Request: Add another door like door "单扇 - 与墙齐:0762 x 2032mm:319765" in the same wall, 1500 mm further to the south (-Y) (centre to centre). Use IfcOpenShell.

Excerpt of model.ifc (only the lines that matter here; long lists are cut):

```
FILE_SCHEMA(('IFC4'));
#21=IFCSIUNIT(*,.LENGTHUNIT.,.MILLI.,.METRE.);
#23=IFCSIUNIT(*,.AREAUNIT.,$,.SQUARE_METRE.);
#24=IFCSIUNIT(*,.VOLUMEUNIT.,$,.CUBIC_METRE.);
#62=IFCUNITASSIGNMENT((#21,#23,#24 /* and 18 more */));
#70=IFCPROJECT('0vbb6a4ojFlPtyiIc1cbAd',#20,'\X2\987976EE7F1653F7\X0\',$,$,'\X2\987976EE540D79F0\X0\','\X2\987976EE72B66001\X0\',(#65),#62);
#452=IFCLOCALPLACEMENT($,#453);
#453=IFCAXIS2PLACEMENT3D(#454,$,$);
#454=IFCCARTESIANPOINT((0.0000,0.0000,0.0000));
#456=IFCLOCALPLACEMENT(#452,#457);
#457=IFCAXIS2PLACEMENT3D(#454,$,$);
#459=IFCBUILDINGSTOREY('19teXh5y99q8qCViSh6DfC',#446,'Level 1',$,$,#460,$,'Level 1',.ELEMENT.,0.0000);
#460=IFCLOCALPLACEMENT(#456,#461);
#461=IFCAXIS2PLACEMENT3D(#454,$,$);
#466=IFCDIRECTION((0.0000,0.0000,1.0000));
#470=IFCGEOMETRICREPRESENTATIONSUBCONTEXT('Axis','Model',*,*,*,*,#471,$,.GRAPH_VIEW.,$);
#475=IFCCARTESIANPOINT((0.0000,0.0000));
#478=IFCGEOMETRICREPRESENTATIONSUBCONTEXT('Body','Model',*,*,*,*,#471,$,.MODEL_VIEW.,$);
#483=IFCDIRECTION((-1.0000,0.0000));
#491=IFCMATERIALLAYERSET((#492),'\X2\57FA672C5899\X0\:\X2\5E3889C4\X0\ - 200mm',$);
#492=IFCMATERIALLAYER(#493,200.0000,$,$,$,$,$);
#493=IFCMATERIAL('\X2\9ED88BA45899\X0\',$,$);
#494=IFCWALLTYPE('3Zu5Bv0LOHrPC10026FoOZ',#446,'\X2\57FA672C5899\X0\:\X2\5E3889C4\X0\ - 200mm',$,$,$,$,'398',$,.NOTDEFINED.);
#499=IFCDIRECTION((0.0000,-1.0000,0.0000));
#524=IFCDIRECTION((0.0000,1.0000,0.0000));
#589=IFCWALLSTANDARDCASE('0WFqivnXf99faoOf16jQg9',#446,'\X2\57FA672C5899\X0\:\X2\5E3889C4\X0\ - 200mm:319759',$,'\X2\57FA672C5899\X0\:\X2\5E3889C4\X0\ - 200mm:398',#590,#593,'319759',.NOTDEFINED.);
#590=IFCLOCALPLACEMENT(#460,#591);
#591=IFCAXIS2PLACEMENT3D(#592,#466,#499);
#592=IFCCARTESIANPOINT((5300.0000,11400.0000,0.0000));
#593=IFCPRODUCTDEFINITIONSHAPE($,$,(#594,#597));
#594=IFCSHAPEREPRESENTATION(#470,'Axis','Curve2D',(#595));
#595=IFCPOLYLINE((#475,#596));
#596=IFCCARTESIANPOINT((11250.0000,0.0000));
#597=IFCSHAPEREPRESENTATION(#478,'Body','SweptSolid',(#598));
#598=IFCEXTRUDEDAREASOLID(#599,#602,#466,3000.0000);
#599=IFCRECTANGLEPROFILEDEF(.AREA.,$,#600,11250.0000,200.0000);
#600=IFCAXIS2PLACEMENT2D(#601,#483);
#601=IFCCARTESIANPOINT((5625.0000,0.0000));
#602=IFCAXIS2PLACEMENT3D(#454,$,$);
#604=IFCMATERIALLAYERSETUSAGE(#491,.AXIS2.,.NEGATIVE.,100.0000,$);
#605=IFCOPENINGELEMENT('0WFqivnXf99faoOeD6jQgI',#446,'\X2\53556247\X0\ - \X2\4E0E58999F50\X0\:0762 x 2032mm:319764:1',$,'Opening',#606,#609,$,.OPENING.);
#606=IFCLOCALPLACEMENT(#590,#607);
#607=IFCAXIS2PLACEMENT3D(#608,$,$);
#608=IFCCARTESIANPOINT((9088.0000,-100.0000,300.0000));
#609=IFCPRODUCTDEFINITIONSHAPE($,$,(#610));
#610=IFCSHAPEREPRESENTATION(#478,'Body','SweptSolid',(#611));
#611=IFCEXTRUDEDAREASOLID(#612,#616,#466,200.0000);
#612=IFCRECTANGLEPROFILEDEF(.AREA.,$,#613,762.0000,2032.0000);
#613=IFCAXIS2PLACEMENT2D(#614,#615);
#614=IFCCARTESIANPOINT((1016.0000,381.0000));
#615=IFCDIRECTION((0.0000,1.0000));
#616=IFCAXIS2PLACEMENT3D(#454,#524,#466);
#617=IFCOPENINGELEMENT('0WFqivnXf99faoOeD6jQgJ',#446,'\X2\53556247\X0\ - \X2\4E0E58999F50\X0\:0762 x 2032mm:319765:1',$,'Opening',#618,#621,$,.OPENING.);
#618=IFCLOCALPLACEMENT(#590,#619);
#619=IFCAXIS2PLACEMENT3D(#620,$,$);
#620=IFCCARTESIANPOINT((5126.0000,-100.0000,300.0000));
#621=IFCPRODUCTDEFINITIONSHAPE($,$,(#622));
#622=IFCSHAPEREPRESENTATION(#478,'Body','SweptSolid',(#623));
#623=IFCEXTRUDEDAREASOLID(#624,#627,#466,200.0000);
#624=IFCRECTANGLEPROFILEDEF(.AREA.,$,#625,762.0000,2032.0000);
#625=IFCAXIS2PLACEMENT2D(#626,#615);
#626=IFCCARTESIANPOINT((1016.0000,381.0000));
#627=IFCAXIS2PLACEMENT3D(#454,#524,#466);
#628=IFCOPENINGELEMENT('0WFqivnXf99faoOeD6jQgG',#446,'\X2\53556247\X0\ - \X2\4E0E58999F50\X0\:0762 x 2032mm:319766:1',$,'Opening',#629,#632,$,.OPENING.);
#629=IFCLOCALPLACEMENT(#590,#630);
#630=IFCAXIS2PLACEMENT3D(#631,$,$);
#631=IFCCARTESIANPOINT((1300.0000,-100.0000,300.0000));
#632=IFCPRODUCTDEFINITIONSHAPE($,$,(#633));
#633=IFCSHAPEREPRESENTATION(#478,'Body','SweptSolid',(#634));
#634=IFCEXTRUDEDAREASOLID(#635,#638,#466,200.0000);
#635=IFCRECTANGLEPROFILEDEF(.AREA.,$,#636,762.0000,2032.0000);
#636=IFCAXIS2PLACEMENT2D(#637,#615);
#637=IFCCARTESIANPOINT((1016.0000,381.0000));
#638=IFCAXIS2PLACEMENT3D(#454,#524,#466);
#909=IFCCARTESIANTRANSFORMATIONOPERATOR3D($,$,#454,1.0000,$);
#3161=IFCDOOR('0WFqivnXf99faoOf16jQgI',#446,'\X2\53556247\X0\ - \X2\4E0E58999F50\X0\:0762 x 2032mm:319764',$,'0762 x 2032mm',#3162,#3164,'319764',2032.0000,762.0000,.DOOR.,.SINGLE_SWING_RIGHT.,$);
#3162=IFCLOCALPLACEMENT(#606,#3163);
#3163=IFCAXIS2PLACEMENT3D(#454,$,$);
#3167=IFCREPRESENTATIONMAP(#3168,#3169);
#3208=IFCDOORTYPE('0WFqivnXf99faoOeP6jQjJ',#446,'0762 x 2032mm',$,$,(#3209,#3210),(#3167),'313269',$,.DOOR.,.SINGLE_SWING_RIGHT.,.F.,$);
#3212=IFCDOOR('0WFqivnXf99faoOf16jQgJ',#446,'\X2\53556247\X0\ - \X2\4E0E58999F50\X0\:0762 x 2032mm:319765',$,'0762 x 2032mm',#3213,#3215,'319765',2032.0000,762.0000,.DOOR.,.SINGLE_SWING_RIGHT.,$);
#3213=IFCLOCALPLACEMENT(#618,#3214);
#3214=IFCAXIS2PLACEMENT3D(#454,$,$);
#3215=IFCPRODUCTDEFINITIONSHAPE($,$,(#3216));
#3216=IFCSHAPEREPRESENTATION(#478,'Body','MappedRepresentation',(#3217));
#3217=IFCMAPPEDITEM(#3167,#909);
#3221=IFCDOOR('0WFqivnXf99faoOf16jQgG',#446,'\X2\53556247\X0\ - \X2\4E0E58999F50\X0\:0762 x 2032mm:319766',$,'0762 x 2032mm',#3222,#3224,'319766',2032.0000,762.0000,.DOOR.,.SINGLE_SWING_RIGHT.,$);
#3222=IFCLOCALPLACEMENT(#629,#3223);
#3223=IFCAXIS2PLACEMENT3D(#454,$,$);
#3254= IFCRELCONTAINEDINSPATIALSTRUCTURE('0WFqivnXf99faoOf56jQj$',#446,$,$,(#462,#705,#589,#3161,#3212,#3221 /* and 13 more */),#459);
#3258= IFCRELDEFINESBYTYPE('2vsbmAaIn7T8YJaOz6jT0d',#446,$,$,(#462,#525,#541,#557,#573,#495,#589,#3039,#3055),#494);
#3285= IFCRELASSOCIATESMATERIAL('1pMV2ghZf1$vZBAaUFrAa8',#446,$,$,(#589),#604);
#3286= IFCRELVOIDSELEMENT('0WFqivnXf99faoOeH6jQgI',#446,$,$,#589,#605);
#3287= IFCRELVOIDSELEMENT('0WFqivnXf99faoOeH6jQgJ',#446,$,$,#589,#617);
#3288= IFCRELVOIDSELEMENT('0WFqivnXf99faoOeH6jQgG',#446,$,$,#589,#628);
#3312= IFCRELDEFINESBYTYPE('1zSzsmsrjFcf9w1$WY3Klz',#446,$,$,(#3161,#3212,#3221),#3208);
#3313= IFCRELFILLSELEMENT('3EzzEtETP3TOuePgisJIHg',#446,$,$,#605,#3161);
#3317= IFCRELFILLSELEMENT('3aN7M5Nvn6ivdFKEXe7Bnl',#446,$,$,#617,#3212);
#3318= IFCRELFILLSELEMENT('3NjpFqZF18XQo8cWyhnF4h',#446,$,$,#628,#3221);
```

```python
import ifcopenshell
import ifcopenshell.api.feature
import ifcopenshell.api.geometry
import ifcopenshell.api.root
import ifcopenshell.geom
import ifcopenshell.util.element
import ifcopenshell.util.placement
import ifcopenshell.util.shape
import ifcopenshell.util.unit

model = ifcopenshell.open("model.ifc")
unit_scale = ifcopenshell.util.unit.calculate_unit_scale(model)
settings = ifcopenshell.geom.settings()


def volume(element):
    """Net volume in cubic metres, openings subtracted."""
    shape = ifcopenshell.geom.create_shape(settings, element)
    return ifcopenshell.util.shape.get_volume(shape.geometry)


def reuse_history(source, copy):
    """copy_class also copies each property set's owner history, people and application; keep the originals."""
    for rel in copy.IsDefinedBy:
        if rel.is_a("IfcRelDefinesByProperties") and (history := rel.RelatingPropertyDefinition.OwnerHistory):
            rel.RelatingPropertyDefinition.OwnerHistory = source.OwnerHistory
            ifcopenshell.util.element.remove_deep2(model, history)


door = model.by_guid("0WFqivnXf99faoOf16jQgJ")
opening = door.FillsVoids[0].RelatingOpeningElement
wall = opening.VoidsElements[0].RelatingBuildingElement
before = volume(wall)
shift = ifcopenshell.util.placement.get_local_placement(wall.ObjectPlacement)[:3, 0] * 1.5 / unit_scale

# copy_class copies the void relationship, type, container and properties, but no geometry.
new_opening = ifcopenshell.api.root.copy_class(model, product=opening)
new_opening.Representation = ifcopenshell.util.element.copy_deep(
    model, opening.Representation, exclude=["IfcGeometricRepresentationContext", "IfcRepresentationMap"]
)
new_opening.Name = "单扇 - 与墙齐:0762 x 2032mm"
new_door = ifcopenshell.api.root.copy_class(model, product=door)
new_door.Representation = ifcopenshell.util.element.copy_deep(
    model, door.Representation, exclude=["IfcGeometricRepresentationContext", "IfcRepresentationMap"]
)
new_door.Name = "单扇 - 与墙齐:0762 x 2032mm"
new_door.Tag = None
reuse_history(door, new_door)
ifcopenshell.api.feature.add_filling(model, opening=new_opening, element=new_door)

for old, new in ((opening, new_opening), (door, new_door)):
    matrix = ifcopenshell.util.placement.get_local_placement(old.ObjectPlacement)
    matrix[:3, 3] += shift
    ifcopenshell.api.geometry.edit_object_placement(model, product=new, matrix=matrix, is_si=False)

after = volume(wall)

print(f"wall volume {before:.3f} -> {after:.3f} m3")

model.write("model_updated.ifc")
```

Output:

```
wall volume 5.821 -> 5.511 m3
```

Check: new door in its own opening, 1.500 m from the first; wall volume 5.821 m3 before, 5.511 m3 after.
